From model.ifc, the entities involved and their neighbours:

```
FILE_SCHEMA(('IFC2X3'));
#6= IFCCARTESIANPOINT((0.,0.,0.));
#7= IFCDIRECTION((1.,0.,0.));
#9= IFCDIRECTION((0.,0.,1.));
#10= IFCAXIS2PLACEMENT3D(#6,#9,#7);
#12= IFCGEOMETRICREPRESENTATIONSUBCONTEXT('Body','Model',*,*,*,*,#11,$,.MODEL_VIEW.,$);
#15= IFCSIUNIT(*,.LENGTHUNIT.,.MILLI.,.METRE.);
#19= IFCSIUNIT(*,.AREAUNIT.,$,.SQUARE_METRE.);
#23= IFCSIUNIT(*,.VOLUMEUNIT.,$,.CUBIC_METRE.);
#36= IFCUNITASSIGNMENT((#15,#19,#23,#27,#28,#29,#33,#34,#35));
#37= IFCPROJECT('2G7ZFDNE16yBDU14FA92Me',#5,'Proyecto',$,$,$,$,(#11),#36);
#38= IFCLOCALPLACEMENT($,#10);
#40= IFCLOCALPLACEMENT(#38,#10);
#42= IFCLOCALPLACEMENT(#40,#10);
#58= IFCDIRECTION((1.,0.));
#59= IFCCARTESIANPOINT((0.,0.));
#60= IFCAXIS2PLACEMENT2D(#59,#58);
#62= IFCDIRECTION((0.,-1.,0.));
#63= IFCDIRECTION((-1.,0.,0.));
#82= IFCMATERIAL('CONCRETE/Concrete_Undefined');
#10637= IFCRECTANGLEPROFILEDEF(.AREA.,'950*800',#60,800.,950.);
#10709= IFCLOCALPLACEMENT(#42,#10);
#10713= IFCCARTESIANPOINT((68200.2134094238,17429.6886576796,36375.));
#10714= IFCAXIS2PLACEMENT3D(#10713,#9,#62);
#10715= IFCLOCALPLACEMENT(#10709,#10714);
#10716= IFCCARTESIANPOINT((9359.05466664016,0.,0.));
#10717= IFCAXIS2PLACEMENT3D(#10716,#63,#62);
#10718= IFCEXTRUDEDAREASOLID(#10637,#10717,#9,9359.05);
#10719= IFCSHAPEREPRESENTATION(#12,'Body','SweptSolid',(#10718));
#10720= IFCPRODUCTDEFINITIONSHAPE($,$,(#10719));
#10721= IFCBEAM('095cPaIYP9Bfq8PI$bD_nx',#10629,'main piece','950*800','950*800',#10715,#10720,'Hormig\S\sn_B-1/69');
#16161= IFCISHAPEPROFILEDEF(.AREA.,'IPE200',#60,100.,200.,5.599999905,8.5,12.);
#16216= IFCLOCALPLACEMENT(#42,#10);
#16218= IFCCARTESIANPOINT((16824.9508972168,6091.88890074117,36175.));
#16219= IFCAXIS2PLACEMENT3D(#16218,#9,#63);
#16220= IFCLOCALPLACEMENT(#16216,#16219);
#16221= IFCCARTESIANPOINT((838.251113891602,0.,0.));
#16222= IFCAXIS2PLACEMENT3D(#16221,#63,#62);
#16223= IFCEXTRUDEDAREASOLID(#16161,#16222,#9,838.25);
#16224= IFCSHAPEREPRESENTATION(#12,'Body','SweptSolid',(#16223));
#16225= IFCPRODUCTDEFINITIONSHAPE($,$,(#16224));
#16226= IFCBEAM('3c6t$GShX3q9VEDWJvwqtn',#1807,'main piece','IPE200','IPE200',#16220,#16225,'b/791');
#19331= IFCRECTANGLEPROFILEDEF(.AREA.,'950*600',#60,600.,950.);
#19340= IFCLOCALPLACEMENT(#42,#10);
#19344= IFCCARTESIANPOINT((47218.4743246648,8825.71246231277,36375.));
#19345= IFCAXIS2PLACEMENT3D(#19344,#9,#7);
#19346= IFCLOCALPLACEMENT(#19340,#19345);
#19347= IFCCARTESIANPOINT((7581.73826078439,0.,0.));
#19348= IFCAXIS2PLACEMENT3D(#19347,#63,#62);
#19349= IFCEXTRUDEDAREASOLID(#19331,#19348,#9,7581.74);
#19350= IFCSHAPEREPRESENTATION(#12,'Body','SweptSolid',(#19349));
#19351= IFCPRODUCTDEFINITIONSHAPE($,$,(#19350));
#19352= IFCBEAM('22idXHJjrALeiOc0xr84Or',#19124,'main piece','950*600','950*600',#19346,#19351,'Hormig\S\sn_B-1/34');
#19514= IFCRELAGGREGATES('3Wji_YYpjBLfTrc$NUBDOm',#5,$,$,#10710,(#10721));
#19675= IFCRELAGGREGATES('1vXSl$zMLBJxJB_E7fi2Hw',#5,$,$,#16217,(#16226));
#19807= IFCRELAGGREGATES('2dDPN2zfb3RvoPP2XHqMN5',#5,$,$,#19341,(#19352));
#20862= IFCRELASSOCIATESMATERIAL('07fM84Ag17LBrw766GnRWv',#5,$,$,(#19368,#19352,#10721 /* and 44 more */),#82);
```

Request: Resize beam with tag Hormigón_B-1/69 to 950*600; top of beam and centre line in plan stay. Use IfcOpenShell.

```python
import ifcopenshell
import ifcopenshell.util.element
import ifcopenshell.util.representation

model = ifcopenshell.open("model.ifc")

member = model.by_id(10721)
source = next(p for p in model.by_type("IfcRectangleProfileDef") if p.ProfileName == "950*600")

body = ifcopenshell.util.representation.get_representation(member, "Model", "Body")
solid = body.Items[0]
old_profile = solid.SweptArea

# Copy the section's sizes but keep this member's own profile position.
profile = ifcopenshell.util.element.copy(model, source)
# Profiles are centred, so shift by half the change in depth to hold the top.
shift = (old_profile.YDim - profile.YDim) / 2
x, y = old_profile.Position.Location.Coordinates
up = (0.0, 1.0)  # upwards, in the solid's own plane
location = model.createIfcCartesianPoint((x + up[0] * shift, y + up[1] * shift))
profile.Position = model.createIfcAxis2Placement2D(location, old_profile.Position.RefDirection)
solid.SweptArea = profile
if not model.get_total_inverses(old_profile):
    ifcopenshell.util.element.remove_deep2(model, old_profile)
member.Description = member.Description.replace("950*800", "950*600")
member.ObjectType = member.ObjectType.replace("950*800", "950*600")

print(solid.SweptArea)

model.write("model_updated.ifc")
```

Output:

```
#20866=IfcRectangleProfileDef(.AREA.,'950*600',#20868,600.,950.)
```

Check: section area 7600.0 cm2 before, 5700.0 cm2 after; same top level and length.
